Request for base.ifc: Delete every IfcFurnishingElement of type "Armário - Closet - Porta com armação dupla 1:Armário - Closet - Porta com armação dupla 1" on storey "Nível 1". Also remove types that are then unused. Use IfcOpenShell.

First a look at what the model holds.

```python
import ifcopenshell
import ifcopenshell.util.element

model = ifcopenshell.open("base.ifc")
print(model.schema)
storey = next(s for s in model.by_type("IfcBuildingStorey") if s.Name == "Nível 1")
furniture = [e for e in ifcopenshell.util.element.get_decomposition(storey) if e.is_a("IfcFurnishingElement")]
seen = {}
for e in furniture:
    element_type = ifcopenshell.util.element.get_type(e)
    name = element_type.Name if element_type not in (None, e) else None
    seen[name] = seen.get(name, 0) + 1
for name, count in sorted(seen.items(), key=str):
    print(count, "x", name)
```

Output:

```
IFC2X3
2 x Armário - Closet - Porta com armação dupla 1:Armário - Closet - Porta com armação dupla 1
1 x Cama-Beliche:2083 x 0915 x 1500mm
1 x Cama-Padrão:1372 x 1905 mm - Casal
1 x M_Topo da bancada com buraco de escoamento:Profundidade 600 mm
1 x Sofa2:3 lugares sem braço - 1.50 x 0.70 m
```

```python
import ifcopenshell
import ifcopenshell.api.root
import ifcopenshell.util.element

model = ifcopenshell.open("base.ifc")

storey = next(s for s in model.by_type("IfcBuildingStorey") if s.Name == "Nível 1")
furniture = [e for e in ifcopenshell.util.element.get_decomposition(storey) if e.is_a("IfcFurnishingElement")]
targets = [e for e in furniture if (t := ifcopenshell.util.element.get_type(e)) not in (None, e) and t.Name == "Armário - Closet - Porta com armação dupla 1:Armário - Closet - Porta com armação dupla 1"]
types = {ifcopenshell.util.element.get_type(e) for e in targets} - {None, *targets}

for e in targets:
    ifcopenshell.api.root.remove_product(model, product=e)
print(len(targets), "removed")

unused = [t for t in types if not ifcopenshell.util.element.get_types(t)]
for t in unused:
    ifcopenshell.api.root.remove_product(model, product=t)
print(len(unused), "unused types removed")

model.write("base_edited.ifc")
```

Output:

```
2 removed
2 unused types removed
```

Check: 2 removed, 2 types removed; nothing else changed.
